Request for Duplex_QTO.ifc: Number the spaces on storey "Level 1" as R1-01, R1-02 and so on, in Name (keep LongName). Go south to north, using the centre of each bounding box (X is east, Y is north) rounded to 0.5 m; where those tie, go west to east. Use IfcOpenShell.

First a look at what the model holds.

```python
import ifcopenshell
import ifcopenshell.util.element
import ifcopenshell.util.placement

model = ifcopenshell.open("Duplex_QTO.ifc")
print(model.schema)
storey = next(s for s in model.by_type("IfcBuildingStorey") if s.Name == "Level 1")
spaces = [e for e in ifcopenshell.util.element.get_decomposition(storey) if e.is_a("IfcSpace")]
for e in sorted(spaces, key=lambda e: e.id()):
    origin = ifcopenshell.util.placement.get_local_placement(e.ObjectPlacement)[:3, 3]
    print(e.id(), e.Name, e.LongName, origin.round(2) + 0.0, sep=" | ")
```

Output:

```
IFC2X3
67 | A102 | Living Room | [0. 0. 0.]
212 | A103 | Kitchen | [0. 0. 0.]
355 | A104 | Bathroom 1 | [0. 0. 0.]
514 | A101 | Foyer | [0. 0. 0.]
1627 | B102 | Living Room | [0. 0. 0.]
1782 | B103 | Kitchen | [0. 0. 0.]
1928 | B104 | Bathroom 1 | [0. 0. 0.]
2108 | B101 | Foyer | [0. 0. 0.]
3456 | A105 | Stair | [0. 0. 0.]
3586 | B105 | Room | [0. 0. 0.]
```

```python
import ifcopenshell
import ifcopenshell.geom
import ifcopenshell.util.element
import ifcopenshell.util.shape

model = ifcopenshell.open("Duplex_QTO.ifc")
settings = ifcopenshell.geom.settings()
settings.set("use-world-coords", True)


def centre(element):
    shape = ifcopenshell.geom.create_shape(settings, element)
    return ifcopenshell.util.shape.get_bbox_centroid(shape.geometry)


storey = next(s for s in model.by_type("IfcBuildingStorey") if s.Name == "Level 1")
spaces = [e for e in ifcopenshell.util.element.get_decomposition(storey) if e.is_a("IfcSpace")]

# Insertion points can sit at a corner or the storey origin, so sort by the geometry (in metres).
centres = {e: centre(e) for e in spaces}
spaces.sort(key=lambda e: (round(centres[e][1] / 0.5), centres[e][0]))

for i, e in enumerate(spaces, start=1):
    number = f"R1-{i:02d}"
    e.Name = number
    print(e.id(), number)

model.write("Duplex_QTO_edited.ifc")
```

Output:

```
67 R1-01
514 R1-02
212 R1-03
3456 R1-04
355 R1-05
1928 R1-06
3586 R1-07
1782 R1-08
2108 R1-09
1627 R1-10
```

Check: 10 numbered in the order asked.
